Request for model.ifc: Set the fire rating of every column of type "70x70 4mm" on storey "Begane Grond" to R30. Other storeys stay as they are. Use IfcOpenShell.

First a look at what the model holds.

```python
import ifcopenshell
import ifcopenshell.util.element

model = ifcopenshell.open("model.ifc")
print(model.schema)
storey = next(s for s in model.by_type("IfcBuildingStorey") if s.Name == "Begane Grond")
columns = [e for e in ifcopenshell.util.element.get_decomposition(storey) if e.is_a("IfcColumn")]
seen = {}
for e in columns:
    element_type = ifcopenshell.util.element.get_type(e)
    key = (element_type.Name if element_type != e and element_type else None, ifcopenshell.util.element.get_pset(e, "Pset_ColumnCommon", "FireRating"))
    seen[key] = seen.get(key, 0) + 1
for (name, value), count in sorted(seen.items(), key=str):
    print(count, "x", name, "|", value)
```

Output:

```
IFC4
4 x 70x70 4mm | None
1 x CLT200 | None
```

```python
import ifcopenshell
import ifcopenshell.api.pset
import ifcopenshell.util.element

model = ifcopenshell.open("model.ifc")

storey = next(s for s in model.by_type("IfcBuildingStorey") if s.Name == "Begane Grond")
columns = [e for e in ifcopenshell.util.element.get_decomposition(storey) if e.is_a("IfcColumn")]

count = 0
for e in columns:
    element_type = ifcopenshell.util.element.get_type(e)
    if element_type in (None, e) or element_type.Name != "70x70 4mm":
        continue
    # add_pset returns the element's existing set when there is one.
    pset = ifcopenshell.api.pset.add_pset(model, product=e, name="Pset_ColumnCommon")
    ifcopenshell.api.pset.edit_pset(model, pset=pset, properties={"FireRating": "R30"})
    count += 1

print(count, "columns updated")

model.write("model-out.ifc")
```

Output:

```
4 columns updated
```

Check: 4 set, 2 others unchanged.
